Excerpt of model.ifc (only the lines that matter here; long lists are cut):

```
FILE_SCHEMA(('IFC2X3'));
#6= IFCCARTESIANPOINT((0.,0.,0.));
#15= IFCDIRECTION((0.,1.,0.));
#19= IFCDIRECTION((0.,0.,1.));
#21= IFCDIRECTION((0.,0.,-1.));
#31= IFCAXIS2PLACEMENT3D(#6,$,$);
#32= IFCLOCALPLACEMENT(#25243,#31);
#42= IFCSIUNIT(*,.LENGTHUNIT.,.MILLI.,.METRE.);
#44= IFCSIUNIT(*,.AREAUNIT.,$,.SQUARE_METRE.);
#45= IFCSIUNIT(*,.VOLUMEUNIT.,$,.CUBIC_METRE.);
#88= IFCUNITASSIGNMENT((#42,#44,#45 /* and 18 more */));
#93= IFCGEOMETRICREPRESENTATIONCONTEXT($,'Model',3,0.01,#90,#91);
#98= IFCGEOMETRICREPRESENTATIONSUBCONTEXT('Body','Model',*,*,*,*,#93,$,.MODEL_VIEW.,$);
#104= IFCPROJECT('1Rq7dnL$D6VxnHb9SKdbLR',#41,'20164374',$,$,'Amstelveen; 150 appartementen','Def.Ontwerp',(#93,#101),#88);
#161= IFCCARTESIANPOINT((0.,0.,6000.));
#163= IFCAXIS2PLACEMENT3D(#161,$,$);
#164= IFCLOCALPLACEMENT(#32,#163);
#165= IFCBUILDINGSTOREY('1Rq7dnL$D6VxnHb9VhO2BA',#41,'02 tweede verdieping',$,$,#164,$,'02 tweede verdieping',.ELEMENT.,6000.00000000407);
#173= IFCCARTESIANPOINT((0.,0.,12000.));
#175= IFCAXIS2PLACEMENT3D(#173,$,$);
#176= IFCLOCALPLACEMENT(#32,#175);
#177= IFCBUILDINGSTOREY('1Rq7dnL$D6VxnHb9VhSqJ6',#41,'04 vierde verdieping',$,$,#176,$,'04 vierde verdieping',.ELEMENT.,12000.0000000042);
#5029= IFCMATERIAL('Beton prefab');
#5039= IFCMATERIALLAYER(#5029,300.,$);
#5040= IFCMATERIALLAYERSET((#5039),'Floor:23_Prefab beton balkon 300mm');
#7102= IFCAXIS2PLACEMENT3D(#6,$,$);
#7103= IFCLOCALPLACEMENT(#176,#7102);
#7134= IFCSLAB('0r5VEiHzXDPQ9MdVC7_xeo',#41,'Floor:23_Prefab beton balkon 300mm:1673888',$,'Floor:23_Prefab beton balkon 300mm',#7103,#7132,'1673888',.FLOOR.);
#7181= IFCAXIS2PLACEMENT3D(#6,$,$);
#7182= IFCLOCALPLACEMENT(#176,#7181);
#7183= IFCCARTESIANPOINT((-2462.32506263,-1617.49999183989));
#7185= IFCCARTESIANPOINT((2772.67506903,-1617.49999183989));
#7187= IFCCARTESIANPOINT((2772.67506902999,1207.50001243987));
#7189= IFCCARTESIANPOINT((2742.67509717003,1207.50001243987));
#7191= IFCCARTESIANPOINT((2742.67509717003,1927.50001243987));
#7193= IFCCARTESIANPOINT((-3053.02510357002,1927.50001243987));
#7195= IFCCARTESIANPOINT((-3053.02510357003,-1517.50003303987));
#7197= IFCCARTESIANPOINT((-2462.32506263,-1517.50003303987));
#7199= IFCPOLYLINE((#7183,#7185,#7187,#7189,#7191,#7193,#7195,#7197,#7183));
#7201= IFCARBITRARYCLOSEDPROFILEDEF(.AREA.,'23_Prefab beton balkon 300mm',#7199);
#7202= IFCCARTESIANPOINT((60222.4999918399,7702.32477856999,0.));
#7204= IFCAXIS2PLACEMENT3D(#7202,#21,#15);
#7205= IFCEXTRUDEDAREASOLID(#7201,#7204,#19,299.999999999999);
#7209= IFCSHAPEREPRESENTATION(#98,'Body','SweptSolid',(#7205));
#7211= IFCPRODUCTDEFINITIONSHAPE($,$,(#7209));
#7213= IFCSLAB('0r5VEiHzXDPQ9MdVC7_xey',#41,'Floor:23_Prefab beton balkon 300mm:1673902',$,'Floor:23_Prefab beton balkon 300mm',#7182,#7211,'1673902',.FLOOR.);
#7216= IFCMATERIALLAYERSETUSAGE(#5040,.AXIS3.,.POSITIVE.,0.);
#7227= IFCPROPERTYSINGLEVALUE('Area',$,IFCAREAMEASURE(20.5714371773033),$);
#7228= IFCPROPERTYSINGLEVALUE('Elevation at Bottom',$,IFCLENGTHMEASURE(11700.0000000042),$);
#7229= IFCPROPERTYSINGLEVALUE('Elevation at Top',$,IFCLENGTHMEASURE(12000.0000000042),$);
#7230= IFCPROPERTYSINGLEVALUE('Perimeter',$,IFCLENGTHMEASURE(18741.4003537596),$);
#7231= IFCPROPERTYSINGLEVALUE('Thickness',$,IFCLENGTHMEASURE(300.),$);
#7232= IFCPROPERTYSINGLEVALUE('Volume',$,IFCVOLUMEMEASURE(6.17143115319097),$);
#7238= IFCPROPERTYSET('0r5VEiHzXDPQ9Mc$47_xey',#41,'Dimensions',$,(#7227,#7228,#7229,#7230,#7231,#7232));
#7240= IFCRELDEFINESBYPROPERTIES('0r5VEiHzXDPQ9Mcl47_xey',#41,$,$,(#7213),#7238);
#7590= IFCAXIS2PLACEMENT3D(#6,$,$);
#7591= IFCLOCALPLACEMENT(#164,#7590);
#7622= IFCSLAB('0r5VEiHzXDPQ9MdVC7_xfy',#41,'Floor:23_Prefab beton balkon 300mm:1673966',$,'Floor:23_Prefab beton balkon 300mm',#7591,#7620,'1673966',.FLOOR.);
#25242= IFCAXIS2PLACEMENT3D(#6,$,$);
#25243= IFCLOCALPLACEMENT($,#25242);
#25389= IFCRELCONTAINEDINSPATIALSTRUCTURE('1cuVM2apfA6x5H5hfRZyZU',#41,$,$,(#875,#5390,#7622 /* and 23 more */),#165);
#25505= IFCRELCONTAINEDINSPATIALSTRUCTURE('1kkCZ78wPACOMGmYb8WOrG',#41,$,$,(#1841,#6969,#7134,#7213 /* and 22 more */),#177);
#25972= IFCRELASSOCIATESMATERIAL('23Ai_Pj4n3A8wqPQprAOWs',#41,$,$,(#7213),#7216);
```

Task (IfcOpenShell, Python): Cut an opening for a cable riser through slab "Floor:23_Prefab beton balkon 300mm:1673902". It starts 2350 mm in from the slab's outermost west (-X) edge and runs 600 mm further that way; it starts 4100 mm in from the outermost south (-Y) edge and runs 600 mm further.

```python
import numpy as np
import ifcopenshell
import ifcopenshell.api.feature
import ifcopenshell.api.geometry
import ifcopenshell.api.pset
import ifcopenshell.api.root
import ifcopenshell.geom
import ifcopenshell.util.element
import ifcopenshell.util.placement
import ifcopenshell.util.representation
import ifcopenshell.util.shape
import ifcopenshell.util.unit

model = ifcopenshell.open("model.ifc")
unit_scale = ifcopenshell.util.unit.calculate_unit_scale(model)
area_scale = ifcopenshell.util.unit.calculate_unit_scale(model, "AREAUNIT")
volume_scale = ifcopenshell.util.unit.calculate_unit_scale(model, "VOLUMEUNIT")
settings = ifcopenshell.geom.settings()


def volume(element):
    """Net volume in cubic metres, openings subtracted."""
    shape = ifcopenshell.geom.create_shape(settings, element)
    return ifcopenshell.util.shape.get_volume(shape.geometry)


slab = model.by_guid("0r5VEiHzXDPQ9MdVC7_xey")
before = volume(slab)

# Extent in the slab's own axes, in metres. The edges named are its -X and -Y sides.
slab_shape = ifcopenshell.geom.create_shape(settings, slab)
vertices = ifcopenshell.util.shape.get_vertices(slab_shape.geometry)
x_min, y_min, bottom = vertices.min(axis=0)
top = vertices[:, 2].max()

opening = ifcopenshell.api.root.create_entity(model, ifc_class="IfcOpeningElement", name="Cable riser opening")
context = ifcopenshell.util.representation.get_context(model, "Model", "Body", "MODEL_VIEW")
width, depth = 0.6, 0.6
outline = [(0.0, 0.0), (width, 0.0), (width, depth), (0.0, depth), (0.0, 0.0)]
# Overshoot both faces by 50 mm so the cut is clean.
shape = ifcopenshell.api.geometry.add_slab_representation(
    model, context=context, depth=top - bottom + 0.1, polyline=outline
)
ifcopenshell.api.geometry.assign_representation(model, product=opening, representation=shape)

matrix = ifcopenshell.util.placement.get_local_placement(slab.ObjectPlacement)
matrix[:, 3] = matrix @ np.append(np.array([x_min + 2.35, y_min + 4.1, bottom - 0.05]) / unit_scale, 1.0)
ifcopenshell.api.geometry.edit_object_placement(model, product=opening, matrix=matrix, is_si=False)
ifcopenshell.api.feature.add_feature(model, feature=opening, element=slab)

after = volume(slab)

# Update the slab's stored quantities.
pset = model.by_id(ifcopenshell.util.element.get_pset(slab, "Dimensions", should_inherit=False)["id"])
ifcopenshell.api.pset.edit_pset(model, pset=pset, properties={
    "Area": model.create_entity("IfcAreaMeasure", after / (top - bottom) / area_scale),
    "Volume": model.create_entity("IfcVolumeMeasure", after / volume_scale),
})

print(f"slab volume {before:.3f} -> {after:.3f} m3")

model.write("model_updated.ifc")
```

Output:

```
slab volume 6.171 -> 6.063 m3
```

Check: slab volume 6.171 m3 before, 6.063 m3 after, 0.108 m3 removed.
